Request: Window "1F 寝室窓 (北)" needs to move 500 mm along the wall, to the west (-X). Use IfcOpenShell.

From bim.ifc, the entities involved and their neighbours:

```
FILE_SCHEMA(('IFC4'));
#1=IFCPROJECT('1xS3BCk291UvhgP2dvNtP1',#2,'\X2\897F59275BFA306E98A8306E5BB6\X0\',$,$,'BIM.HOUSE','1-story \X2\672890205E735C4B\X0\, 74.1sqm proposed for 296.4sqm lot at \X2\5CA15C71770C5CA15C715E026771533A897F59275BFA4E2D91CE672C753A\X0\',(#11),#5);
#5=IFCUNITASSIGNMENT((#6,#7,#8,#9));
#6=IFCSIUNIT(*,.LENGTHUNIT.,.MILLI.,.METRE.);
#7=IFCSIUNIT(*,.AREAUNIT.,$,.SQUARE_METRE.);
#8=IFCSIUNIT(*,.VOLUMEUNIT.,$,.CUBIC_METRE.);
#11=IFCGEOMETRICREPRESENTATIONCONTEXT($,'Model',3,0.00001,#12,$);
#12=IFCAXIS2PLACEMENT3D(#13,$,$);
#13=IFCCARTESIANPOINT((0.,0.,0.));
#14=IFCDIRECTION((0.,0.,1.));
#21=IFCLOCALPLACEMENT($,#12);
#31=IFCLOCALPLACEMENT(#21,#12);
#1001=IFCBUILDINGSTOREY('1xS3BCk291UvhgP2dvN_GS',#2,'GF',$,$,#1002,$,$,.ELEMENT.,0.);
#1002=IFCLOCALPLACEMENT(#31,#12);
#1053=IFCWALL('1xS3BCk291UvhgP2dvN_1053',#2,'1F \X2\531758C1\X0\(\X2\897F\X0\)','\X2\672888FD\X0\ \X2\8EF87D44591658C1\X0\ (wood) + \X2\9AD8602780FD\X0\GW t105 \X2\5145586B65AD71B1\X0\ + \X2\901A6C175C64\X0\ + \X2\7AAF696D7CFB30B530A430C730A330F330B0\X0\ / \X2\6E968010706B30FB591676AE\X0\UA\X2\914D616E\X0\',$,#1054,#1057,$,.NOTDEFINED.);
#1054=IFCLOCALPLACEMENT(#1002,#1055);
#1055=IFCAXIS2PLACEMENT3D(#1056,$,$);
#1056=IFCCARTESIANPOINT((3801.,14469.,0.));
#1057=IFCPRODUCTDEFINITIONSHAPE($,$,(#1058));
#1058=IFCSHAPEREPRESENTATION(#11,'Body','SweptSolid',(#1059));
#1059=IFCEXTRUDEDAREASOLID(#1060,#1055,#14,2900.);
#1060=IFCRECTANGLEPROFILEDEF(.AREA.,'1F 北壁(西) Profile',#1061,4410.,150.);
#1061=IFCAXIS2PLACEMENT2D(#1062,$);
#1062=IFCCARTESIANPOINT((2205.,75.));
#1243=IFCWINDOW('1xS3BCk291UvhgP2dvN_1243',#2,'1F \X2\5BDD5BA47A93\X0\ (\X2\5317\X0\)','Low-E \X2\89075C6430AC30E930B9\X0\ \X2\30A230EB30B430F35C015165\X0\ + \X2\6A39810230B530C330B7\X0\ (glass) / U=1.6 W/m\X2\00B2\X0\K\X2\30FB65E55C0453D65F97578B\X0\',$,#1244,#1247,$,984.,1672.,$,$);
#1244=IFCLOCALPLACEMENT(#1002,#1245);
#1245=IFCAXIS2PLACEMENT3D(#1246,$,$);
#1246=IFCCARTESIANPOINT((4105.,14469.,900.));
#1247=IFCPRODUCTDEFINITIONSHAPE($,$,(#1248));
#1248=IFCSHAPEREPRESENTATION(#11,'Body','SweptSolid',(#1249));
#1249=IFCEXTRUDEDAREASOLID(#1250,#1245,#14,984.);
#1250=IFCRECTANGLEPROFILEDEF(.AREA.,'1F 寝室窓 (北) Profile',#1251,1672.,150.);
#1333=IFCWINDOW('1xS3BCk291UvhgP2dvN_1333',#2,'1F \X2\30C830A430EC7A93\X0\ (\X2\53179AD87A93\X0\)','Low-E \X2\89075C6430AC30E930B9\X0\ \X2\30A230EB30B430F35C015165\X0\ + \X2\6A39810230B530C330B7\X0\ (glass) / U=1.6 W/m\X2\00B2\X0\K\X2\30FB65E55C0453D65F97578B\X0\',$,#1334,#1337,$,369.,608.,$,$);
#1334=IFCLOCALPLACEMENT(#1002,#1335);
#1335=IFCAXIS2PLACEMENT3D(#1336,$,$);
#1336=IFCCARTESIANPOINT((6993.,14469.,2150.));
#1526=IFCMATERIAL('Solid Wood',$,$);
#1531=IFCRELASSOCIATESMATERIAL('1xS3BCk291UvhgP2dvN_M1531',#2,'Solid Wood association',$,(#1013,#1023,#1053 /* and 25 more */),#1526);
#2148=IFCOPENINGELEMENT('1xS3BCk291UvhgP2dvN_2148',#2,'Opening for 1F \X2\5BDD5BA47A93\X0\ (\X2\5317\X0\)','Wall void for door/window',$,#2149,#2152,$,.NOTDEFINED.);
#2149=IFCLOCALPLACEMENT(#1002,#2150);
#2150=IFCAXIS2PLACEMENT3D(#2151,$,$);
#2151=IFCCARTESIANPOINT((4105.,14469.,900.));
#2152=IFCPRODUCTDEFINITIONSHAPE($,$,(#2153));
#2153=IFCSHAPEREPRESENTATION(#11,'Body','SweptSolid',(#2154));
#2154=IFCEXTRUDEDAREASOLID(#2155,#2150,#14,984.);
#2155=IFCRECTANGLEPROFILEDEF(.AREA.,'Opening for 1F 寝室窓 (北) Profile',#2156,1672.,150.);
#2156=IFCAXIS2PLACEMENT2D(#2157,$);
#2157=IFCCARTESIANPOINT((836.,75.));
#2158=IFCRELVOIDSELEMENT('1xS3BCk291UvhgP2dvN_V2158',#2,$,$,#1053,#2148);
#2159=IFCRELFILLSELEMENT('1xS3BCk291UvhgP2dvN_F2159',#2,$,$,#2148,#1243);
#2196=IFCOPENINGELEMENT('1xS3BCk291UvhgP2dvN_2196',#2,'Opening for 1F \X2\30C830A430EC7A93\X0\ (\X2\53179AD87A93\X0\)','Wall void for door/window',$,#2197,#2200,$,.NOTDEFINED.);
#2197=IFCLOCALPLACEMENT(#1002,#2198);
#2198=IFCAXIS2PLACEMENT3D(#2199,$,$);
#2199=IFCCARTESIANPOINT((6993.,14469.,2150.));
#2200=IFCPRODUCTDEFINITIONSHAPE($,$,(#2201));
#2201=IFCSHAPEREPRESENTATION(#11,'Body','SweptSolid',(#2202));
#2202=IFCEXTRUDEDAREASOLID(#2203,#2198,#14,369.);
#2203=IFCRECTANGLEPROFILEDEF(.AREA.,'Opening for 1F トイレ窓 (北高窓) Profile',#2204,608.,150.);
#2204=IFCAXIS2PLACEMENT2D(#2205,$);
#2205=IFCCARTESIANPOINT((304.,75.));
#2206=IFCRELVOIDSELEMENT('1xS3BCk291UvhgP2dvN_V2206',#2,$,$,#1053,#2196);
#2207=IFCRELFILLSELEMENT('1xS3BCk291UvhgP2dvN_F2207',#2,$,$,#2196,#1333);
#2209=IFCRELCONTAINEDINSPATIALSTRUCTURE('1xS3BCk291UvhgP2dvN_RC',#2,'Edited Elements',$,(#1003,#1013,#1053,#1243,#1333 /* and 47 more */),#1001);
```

```python
import ifcopenshell
import ifcopenshell.api.geometry
import ifcopenshell.util.placement

model = ifcopenshell.open("bim.ifc")

window = model.by_guid("1xS3BCk291UvhgP2dvN_1243")
opening = window.FillsVoids[0].RelatingOpeningElement
wall = opening.VoidsElements[0].RelatingBuildingElement

wall_matrix = ifcopenshell.util.placement.get_local_placement(wall.ObjectPlacement)
shift = wall_matrix[:3, 0] * -500.0
before = ifcopenshell.util.placement.get_local_placement(window.ObjectPlacement)[:3, 3].copy()

# The window is not placed relative to its opening, so move both.
for product in (opening, window):
    matrix = ifcopenshell.util.placement.get_local_placement(product.ObjectPlacement)
    matrix[:3, 3] += shift
    ifcopenshell.api.geometry.edit_object_placement(model, product=product, matrix=matrix, is_si=False)

after = ifcopenshell.util.placement.get_local_placement(window.ObjectPlacement)[:3, 3]
print("window moved by", (after - before).round(3) + 0.0)

model.write("bim_edited.ifc")
```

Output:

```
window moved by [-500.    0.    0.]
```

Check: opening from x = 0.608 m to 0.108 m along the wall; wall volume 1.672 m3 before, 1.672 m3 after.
